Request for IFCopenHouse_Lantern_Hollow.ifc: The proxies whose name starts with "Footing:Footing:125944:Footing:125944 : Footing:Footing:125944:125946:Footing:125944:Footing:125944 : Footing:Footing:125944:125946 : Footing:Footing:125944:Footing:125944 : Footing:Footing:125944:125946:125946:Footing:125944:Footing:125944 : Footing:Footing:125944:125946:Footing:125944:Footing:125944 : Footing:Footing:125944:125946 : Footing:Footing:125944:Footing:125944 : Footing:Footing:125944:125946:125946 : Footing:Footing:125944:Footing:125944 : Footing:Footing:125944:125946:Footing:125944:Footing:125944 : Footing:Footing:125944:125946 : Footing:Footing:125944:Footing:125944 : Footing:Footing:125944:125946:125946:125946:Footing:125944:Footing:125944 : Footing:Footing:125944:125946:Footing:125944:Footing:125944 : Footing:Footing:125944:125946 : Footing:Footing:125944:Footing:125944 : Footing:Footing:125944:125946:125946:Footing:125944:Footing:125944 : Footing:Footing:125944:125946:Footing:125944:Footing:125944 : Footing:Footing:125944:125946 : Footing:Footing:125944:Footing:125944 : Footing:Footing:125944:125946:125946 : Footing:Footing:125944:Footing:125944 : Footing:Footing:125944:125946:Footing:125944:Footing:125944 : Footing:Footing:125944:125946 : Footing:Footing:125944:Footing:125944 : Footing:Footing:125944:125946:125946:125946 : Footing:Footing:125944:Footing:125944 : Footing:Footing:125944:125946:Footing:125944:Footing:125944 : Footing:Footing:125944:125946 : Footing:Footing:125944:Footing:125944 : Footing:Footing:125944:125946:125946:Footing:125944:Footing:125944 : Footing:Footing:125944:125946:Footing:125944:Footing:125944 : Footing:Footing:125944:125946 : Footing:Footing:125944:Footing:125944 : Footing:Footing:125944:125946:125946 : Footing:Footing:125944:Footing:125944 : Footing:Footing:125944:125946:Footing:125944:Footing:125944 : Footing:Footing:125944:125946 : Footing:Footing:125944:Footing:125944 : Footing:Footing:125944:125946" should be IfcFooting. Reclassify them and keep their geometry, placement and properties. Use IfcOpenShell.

First a look at what the model holds.

```python
import re

import ifcopenshell

model = ifcopenshell.open("IFCopenHouse_Lantern_Hollow.ifc")
print(model.schema)
seen = {}
for e in model.by_type("IfcBuildingElementProxy"):
    name = re.sub(r":\d+(:\d+)?$", "", e.Name or "")  # drop the element id that some exporters append
    seen[name] = seen.get(name, 0) + 1
for name, count in sorted(seen.items()):
    print(count, "x", name)
```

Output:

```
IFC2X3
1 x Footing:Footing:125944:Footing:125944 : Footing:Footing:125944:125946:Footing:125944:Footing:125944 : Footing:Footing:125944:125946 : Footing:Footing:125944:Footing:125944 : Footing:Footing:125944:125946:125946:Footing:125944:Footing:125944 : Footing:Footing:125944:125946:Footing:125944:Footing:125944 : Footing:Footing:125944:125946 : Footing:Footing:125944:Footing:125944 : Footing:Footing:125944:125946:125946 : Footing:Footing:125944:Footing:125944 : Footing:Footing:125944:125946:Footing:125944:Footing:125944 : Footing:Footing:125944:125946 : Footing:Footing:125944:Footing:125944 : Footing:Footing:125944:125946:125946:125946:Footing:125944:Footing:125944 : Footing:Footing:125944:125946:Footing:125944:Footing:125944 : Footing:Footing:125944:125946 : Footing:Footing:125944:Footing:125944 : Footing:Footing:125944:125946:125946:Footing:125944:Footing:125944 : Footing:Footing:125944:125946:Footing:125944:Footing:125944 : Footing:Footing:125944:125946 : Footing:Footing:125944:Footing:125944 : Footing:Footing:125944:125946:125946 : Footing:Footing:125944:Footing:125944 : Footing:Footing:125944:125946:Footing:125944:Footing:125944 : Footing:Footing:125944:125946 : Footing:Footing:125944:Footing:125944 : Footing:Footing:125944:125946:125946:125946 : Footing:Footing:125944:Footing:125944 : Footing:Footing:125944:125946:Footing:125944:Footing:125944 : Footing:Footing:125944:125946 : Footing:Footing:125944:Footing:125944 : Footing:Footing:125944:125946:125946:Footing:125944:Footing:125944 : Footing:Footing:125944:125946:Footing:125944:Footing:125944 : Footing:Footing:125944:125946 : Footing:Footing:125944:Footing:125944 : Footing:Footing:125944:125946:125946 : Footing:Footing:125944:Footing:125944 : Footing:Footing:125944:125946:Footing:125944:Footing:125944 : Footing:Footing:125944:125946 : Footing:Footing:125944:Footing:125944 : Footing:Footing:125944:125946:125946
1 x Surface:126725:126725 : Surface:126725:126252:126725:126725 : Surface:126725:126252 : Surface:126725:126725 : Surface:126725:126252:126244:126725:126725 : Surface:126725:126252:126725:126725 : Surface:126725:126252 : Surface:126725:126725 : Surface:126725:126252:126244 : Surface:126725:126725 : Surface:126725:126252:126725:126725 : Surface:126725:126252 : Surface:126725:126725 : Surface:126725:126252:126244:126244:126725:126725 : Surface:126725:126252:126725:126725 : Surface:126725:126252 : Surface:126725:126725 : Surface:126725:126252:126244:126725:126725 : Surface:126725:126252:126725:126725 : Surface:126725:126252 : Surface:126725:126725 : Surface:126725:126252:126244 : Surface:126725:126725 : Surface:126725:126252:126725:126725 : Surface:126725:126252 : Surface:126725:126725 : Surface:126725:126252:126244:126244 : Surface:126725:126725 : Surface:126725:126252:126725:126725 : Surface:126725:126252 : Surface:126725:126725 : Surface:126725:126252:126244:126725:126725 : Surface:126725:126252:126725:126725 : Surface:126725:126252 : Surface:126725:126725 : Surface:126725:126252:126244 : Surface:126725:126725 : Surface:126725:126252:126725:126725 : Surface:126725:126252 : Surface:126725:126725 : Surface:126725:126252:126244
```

```python
import ifcopenshell
import ifcopenshell.api.root

model = ifcopenshell.open("IFCopenHouse_Lantern_Hollow.ifc")

proxies = [e.id() for e in model.by_type("IfcBuildingElementProxy") if (e.Name or "").startswith("Footing:Footing:125944:Footing:125944 : Footing:Footing:125944:125946:Footing:125944:Footing:125944 : Footing:Footing:125944:125946 : Footing:Footing:125944:Footing:125944 : Footing:Footing:125944:125946:125946:Footing:125944:Footing:125944 : Footing:Footing:125944:125946:Footing:125944:Footing:125944 : Footing:Footing:125944:125946 : Footing:Footing:125944:Footing:125944 : Footing:Footing:125944:125946:125946 : Footing:Footing:125944:Footing:125944 : Footing:Footing:125944:125946:Footing:125944:Footing:125944 : Footing:Footing:125944:125946 : Footing:Footing:125944:Footing:125944 : Footing:Footing:125944:125946:125946:125946:Footing:125944:Footing:125944 : Footing:Footing:125944:125946:Footing:125944:Footing:125944 : Footing:Footing:125944:125946 : Footing:Footing:125944:Footing:125944 : Footing:Footing:125944:125946:125946:Footing:125944:Footing:125944 : Footing:Footing:125944:125946:Footing:125944:Footing:125944 : Footing:Footing:125944:125946 : Footing:Footing:125944:Footing:125944 : Footing:Footing:125944:125946:125946 : Footing:Footing:125944:Footing:125944 : Footing:Footing:125944:125946:Footing:125944:Footing:125944 : Footing:Footing:125944:125946 : Footing:Footing:125944:Footing:125944 : Footing:Footing:125944:125946:125946:125946 : Footing:Footing:125944:Footing:125944 : Footing:Footing:125944:125946:Footing:125944:Footing:125944 : Footing:Footing:125944:125946 : Footing:Footing:125944:Footing:125944 : Footing:Footing:125944:125946:125946:Footing:125944:Footing:125944 : Footing:Footing:125944:125946:Footing:125944:Footing:125944 : Footing:Footing:125944:125946 : Footing:Footing:125944:Footing:125944 : Footing:Footing:125944:125946:125946 : Footing:Footing:125944:Footing:125944 : Footing:Footing:125944:125946:Footing:125944:Footing:125944 : Footing:Footing:125944:125946 : Footing:Footing:125944:Footing:125944 : Footing:Footing:125944:125946")]
for step_id in proxies:
    proxy = model.by_id(step_id)
    ifcopenshell.api.root.reassign_class(model, product=proxy, ifc_class="IfcFooting", predefined_type="NOTDEFINED")

print(sum(model.by_id(i).is_a("IfcFooting") for i in proxies), "reclassified")

model.write("IFCopenHouse_Lantern_Hollow_edited.ifc")
```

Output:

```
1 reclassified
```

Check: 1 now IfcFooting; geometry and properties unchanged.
